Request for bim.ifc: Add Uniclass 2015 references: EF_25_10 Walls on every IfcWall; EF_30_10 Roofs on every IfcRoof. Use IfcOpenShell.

First a look at what the model holds.

```python
import ifcopenshell

model = ifcopenshell.open("bim.ifc")
print(model.schema)
print("classifications:", [c.Name for c in model.by_type("IfcClassification")])
for ifc_class in ("IfcDoor", "IfcRoof", "IfcStair", "IfcWall", "IfcWindow"):
    print(ifc_class, len(model.by_type(ifc_class)))
```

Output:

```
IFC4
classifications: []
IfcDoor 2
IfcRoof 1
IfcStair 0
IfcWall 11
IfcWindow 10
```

```python
import ifcopenshell
import ifcopenshell.api.classification

model = ifcopenshell.open("bim.ifc")

system = ifcopenshell.api.classification.add_classification(model, classification="Uniclass 2015")

codes = {
    "IfcWall": ("EF_25_10", "Walls"),
    "IfcRoof": ("EF_30_10", "Roofs"),
}
for ifc_class, (code, name) in codes.items():
    products = model.by_type(ifc_class)
    ifcopenshell.api.classification.add_reference(
        model, products=products, classification=system, identification=code, name=name
    )
    print(code, len(products))

model.write("bim-out.ifc")
```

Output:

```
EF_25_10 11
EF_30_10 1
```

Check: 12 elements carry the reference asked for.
